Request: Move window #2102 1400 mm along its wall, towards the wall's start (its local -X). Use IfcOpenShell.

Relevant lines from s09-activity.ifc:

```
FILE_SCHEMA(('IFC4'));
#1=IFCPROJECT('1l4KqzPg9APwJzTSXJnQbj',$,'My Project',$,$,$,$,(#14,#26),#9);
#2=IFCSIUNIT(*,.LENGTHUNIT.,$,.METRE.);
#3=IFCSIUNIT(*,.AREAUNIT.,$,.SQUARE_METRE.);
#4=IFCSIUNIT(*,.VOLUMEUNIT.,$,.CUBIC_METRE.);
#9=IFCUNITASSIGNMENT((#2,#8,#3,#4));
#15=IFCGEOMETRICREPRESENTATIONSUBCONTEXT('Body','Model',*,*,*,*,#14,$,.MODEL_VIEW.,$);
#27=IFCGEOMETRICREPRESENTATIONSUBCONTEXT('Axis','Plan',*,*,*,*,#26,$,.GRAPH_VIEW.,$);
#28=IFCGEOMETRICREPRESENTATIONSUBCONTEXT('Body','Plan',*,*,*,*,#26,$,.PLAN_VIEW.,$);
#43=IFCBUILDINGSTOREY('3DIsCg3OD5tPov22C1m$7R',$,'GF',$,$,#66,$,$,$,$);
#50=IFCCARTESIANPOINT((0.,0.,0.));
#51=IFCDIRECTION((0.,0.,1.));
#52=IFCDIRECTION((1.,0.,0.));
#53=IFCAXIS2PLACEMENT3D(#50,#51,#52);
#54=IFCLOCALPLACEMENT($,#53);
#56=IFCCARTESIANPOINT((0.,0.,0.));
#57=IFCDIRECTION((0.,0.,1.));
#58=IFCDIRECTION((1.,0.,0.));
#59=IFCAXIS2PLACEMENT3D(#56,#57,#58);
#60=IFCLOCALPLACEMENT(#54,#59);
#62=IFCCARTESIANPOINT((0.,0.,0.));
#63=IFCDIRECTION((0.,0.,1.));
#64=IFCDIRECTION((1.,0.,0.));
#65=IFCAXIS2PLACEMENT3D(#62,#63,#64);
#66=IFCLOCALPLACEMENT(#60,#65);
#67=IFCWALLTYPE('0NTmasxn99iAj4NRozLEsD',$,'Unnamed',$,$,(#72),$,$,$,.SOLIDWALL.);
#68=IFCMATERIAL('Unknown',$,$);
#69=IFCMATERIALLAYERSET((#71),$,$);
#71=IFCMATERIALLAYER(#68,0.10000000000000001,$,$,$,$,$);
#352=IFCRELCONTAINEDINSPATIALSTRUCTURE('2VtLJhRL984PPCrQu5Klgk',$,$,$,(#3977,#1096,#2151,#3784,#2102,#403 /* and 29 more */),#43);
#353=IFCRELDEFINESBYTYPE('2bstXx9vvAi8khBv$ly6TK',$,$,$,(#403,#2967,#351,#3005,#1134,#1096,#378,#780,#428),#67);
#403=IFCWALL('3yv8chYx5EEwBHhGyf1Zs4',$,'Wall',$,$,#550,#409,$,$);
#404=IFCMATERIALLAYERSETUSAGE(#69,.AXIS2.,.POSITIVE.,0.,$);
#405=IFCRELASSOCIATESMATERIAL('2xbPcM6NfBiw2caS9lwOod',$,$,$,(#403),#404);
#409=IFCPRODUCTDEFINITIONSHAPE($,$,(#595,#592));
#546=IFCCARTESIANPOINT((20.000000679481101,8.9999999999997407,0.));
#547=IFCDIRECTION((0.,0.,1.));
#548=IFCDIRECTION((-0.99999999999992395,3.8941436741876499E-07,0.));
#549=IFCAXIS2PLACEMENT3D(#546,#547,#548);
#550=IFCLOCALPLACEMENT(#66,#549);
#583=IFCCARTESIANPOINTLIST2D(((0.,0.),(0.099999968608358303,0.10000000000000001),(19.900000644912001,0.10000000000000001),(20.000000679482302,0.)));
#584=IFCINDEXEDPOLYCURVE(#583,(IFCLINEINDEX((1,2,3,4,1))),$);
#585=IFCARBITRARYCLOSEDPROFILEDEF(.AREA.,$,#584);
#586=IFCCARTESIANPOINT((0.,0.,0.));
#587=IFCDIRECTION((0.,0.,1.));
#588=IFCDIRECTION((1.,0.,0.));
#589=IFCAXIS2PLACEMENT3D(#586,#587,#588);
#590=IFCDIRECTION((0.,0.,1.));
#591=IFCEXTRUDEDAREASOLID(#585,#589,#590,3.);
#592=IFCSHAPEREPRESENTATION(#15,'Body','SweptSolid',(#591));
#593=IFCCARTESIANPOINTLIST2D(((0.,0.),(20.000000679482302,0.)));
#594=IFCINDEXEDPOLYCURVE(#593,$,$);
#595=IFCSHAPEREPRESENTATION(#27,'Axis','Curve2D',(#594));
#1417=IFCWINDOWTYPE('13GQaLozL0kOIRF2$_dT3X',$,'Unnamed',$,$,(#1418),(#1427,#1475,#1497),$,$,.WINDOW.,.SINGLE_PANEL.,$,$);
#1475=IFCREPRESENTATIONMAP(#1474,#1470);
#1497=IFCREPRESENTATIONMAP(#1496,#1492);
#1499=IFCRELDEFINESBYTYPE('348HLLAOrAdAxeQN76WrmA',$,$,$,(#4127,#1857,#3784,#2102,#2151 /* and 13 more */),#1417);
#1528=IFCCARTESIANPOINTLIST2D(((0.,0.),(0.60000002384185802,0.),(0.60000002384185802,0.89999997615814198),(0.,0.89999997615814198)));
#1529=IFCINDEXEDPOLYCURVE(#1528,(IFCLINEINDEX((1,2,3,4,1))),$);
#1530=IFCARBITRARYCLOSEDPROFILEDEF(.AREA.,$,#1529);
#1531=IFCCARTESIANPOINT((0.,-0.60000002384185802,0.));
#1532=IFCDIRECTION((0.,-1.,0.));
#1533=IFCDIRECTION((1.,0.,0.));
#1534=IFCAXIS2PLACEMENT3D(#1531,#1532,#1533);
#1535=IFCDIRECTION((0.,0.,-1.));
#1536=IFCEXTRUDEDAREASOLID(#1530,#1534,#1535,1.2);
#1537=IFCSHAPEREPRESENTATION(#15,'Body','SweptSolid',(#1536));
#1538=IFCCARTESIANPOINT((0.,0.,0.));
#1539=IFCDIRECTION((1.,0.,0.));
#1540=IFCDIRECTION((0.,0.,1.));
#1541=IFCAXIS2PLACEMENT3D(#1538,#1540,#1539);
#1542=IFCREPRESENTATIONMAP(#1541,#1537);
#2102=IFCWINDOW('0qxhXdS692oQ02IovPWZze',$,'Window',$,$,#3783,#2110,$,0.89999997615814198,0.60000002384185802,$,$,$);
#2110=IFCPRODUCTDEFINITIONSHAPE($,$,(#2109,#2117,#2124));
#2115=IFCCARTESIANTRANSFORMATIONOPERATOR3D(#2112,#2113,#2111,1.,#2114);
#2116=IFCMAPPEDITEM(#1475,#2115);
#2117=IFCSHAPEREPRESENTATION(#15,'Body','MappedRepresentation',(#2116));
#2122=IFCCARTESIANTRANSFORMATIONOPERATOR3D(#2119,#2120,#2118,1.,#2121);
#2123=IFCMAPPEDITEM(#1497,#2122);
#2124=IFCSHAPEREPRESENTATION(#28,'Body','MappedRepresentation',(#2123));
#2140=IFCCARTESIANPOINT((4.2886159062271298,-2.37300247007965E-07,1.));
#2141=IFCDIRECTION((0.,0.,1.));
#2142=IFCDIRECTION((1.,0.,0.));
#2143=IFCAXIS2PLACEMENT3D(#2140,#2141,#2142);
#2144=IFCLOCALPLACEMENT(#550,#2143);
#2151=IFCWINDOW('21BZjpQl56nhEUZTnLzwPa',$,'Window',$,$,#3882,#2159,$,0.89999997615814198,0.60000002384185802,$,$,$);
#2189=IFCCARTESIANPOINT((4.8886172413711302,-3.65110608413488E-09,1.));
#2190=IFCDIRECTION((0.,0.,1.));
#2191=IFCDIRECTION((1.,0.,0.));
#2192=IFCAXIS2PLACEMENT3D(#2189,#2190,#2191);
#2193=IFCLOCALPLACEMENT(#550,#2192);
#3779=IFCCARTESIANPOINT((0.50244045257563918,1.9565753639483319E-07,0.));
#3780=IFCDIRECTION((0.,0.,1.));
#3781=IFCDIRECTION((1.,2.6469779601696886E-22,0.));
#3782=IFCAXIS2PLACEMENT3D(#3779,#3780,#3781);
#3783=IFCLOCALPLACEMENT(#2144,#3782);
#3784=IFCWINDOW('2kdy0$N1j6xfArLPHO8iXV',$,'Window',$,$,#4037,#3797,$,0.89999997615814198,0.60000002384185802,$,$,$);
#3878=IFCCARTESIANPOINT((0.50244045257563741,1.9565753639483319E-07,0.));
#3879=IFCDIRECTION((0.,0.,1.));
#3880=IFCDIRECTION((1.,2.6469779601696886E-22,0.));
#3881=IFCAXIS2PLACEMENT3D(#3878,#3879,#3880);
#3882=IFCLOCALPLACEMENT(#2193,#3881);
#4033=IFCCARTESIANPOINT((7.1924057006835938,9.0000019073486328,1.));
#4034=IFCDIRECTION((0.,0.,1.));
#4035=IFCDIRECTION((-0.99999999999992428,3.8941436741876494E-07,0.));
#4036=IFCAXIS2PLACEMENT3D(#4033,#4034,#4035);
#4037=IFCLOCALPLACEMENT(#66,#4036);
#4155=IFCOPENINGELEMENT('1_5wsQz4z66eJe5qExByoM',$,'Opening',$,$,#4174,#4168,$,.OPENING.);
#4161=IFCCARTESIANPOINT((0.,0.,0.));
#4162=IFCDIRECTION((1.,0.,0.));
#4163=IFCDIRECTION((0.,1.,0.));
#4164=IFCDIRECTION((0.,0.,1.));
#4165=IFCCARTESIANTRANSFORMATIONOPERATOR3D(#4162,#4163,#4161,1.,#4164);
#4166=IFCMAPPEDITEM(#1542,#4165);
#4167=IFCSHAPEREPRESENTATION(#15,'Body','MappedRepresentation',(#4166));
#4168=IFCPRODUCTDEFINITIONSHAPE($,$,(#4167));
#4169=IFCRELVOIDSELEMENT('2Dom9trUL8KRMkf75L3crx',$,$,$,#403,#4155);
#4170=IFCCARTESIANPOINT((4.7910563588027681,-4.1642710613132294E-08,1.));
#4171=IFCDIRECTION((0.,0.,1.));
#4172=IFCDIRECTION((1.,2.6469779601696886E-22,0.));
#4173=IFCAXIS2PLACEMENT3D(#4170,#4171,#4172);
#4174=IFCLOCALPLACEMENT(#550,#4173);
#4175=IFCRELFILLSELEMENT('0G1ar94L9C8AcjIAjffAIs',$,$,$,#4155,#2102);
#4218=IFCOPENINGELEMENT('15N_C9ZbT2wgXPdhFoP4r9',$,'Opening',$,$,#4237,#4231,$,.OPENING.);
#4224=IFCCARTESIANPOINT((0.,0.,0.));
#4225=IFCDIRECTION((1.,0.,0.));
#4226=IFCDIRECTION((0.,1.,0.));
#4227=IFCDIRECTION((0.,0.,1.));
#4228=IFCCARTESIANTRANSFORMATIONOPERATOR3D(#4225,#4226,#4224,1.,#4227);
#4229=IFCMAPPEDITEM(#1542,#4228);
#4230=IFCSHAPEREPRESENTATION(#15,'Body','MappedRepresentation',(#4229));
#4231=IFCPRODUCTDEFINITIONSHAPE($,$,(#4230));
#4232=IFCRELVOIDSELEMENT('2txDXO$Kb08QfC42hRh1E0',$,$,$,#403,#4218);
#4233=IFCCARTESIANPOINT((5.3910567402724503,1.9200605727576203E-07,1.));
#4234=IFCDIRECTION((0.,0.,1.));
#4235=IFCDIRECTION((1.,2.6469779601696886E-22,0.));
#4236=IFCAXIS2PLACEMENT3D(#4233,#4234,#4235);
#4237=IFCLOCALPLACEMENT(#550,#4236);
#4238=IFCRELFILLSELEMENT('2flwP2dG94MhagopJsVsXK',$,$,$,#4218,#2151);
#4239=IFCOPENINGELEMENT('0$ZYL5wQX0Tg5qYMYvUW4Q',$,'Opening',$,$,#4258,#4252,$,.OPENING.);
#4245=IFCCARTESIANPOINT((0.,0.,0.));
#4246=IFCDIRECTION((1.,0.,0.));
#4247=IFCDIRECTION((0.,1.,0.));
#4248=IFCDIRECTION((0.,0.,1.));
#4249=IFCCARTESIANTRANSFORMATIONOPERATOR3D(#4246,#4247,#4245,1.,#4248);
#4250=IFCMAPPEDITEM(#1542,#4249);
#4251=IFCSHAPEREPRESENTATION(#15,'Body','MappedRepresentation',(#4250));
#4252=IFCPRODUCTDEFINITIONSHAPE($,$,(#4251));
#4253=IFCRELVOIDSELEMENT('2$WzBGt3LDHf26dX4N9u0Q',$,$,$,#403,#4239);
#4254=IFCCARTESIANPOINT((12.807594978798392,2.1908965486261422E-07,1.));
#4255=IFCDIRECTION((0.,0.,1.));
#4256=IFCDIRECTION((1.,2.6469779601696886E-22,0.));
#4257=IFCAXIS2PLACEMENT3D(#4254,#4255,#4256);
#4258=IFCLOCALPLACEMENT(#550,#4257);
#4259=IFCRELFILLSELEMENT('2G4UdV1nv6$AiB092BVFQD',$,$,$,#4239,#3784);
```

```python
import ifcopenshell
import ifcopenshell.api.geometry
import ifcopenshell.util.placement
import ifcopenshell.util.unit

model = ifcopenshell.open("s09-activity.ifc")
unit_scale = ifcopenshell.util.unit.calculate_unit_scale(model)

window = model.by_id(2102)
opening = window.FillsVoids[0].RelatingOpeningElement
wall = opening.VoidsElements[0].RelatingBuildingElement

wall_matrix = ifcopenshell.util.placement.get_local_placement(wall.ObjectPlacement)
shift = wall_matrix[:3, 0] * -1.4 / unit_scale
before = ifcopenshell.util.placement.get_local_placement(window.ObjectPlacement)[:3, 3].copy()

# The window is not placed relative to its opening, so move both.
for product in (opening, window):
    matrix = ifcopenshell.util.placement.get_local_placement(product.ObjectPlacement)
    matrix[:3, 3] += shift
    ifcopenshell.api.geometry.edit_object_placement(model, product=product, matrix=matrix, is_si=False)

after = ifcopenshell.util.placement.get_local_placement(window.ObjectPlacement)[:3, 3]
print("window moved by", (after - before).round(3) + 0.0)

model.write("s09-activity_updated.ifc")
```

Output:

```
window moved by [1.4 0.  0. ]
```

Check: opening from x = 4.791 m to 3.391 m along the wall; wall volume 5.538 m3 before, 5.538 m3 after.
